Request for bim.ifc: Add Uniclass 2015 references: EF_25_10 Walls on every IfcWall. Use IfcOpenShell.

First a look at what the model holds.

```python
import ifcopenshell

model = ifcopenshell.open("bim.ifc")
print(model.schema)
print("classifications:", [c.Name for c in model.by_type("IfcClassification")])
for ifc_class in ("IfcDoor", "IfcRoof", "IfcStair", "IfcWall", "IfcWindow"):
    print(ifc_class, len(model.by_type(ifc_class)))
```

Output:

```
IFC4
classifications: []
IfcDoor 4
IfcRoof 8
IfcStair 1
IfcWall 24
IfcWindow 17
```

```python
import ifcopenshell
import ifcopenshell.api.classification

model = ifcopenshell.open("bim.ifc")

system = ifcopenshell.api.classification.add_classification(model, classification="Uniclass 2015")

codes = {
    "IfcWall": ("EF_25_10", "Walls"),
}
for ifc_class, (code, name) in codes.items():
    products = model.by_type(ifc_class)
    ifcopenshell.api.classification.add_reference(
        model, products=products, classification=system, identification=code, name=name
    )
    print(code, len(products))

model.write("bim_v2.ifc")
```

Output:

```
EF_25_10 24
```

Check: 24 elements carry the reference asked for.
